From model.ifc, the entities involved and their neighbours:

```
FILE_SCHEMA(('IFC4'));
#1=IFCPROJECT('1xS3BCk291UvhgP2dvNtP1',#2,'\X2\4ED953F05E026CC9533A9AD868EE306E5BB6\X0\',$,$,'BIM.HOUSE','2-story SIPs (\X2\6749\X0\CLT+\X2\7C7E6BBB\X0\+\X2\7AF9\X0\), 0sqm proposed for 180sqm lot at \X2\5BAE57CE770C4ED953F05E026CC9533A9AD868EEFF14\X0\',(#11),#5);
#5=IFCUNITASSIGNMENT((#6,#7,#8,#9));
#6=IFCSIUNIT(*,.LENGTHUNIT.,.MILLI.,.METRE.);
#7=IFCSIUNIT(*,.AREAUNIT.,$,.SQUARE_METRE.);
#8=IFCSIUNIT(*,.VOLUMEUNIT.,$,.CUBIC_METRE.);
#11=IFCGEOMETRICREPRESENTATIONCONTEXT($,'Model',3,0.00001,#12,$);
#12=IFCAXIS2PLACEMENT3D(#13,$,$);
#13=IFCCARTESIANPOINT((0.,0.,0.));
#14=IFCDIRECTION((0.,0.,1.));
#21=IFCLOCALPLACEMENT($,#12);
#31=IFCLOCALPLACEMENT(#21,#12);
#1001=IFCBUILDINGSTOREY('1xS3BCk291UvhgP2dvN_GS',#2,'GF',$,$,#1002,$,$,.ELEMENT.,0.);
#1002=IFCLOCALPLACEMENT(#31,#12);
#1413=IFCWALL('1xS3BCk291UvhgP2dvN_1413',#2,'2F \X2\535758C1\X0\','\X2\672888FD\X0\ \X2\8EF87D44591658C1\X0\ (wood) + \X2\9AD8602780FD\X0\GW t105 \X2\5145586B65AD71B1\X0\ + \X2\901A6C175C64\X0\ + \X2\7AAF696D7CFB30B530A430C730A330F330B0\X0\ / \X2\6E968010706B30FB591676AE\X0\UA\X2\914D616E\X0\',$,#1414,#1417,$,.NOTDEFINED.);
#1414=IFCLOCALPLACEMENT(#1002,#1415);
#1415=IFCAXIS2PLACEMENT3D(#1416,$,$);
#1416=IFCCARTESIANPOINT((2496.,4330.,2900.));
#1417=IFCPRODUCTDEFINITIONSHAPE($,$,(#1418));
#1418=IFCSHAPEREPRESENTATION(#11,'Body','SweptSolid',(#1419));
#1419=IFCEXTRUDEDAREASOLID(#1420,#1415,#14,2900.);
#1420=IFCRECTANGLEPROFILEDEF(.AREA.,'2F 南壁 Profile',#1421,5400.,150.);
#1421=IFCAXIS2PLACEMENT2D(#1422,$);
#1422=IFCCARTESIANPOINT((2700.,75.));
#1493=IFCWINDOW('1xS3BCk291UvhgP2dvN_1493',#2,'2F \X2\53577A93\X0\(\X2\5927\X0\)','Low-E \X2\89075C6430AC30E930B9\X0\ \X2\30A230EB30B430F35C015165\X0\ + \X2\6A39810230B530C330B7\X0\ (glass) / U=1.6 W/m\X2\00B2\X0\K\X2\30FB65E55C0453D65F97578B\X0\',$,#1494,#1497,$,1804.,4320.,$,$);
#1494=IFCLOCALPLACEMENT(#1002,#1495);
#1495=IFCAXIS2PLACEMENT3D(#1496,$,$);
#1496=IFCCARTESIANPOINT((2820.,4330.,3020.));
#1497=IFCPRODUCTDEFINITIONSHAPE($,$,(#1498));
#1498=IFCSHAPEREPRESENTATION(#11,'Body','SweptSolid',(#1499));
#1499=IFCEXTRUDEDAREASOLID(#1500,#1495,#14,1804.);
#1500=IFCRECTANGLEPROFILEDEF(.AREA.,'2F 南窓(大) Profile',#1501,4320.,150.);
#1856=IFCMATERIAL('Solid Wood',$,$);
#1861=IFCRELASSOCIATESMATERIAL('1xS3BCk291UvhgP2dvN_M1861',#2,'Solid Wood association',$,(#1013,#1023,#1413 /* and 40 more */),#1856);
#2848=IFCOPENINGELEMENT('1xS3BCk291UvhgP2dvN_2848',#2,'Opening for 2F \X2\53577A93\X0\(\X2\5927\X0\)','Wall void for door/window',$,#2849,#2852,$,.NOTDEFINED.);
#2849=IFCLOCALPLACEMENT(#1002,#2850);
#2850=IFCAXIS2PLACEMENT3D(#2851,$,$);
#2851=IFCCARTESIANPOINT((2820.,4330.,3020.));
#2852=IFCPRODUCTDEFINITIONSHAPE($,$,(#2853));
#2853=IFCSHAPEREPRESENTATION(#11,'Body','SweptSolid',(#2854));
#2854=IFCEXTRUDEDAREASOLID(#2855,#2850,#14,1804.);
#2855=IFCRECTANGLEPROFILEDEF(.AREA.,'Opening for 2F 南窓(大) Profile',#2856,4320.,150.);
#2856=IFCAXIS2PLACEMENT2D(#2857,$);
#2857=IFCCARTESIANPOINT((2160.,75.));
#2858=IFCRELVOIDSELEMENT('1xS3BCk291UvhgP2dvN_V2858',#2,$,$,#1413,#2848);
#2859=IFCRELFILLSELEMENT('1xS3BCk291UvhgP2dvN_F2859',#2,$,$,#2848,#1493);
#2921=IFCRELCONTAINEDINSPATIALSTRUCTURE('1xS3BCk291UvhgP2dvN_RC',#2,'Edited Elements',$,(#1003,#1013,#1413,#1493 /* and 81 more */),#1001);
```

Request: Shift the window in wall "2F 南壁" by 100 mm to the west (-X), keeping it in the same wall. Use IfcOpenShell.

```python
import ifcopenshell
import ifcopenshell.api.geometry
import ifcopenshell.util.placement
import ifcopenshell.util.unit

model = ifcopenshell.open("model.ifc")
unit_scale = ifcopenshell.util.unit.calculate_unit_scale(model)

window = model.by_id(1493)
opening = window.FillsVoids[0].RelatingOpeningElement
wall = opening.VoidsElements[0].RelatingBuildingElement

wall_matrix = ifcopenshell.util.placement.get_local_placement(wall.ObjectPlacement)
shift = wall_matrix[:3, 0] * -0.1 / unit_scale
before = ifcopenshell.util.placement.get_local_placement(window.ObjectPlacement)[:3, 3].copy()

# The window is not placed relative to its opening, so move both.
for product in (opening, window):
    matrix = ifcopenshell.util.placement.get_local_placement(product.ObjectPlacement)
    matrix[:3, 3] += shift
    ifcopenshell.api.geometry.edit_object_placement(model, product=product, matrix=matrix, is_si=False)

after = ifcopenshell.util.placement.get_local_placement(window.ObjectPlacement)[:3, 3]
print("window moved by", (after - before).round(3) + 0.0)

model.write("model-out.ifc")
```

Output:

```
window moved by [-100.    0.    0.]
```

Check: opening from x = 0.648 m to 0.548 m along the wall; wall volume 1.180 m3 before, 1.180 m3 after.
